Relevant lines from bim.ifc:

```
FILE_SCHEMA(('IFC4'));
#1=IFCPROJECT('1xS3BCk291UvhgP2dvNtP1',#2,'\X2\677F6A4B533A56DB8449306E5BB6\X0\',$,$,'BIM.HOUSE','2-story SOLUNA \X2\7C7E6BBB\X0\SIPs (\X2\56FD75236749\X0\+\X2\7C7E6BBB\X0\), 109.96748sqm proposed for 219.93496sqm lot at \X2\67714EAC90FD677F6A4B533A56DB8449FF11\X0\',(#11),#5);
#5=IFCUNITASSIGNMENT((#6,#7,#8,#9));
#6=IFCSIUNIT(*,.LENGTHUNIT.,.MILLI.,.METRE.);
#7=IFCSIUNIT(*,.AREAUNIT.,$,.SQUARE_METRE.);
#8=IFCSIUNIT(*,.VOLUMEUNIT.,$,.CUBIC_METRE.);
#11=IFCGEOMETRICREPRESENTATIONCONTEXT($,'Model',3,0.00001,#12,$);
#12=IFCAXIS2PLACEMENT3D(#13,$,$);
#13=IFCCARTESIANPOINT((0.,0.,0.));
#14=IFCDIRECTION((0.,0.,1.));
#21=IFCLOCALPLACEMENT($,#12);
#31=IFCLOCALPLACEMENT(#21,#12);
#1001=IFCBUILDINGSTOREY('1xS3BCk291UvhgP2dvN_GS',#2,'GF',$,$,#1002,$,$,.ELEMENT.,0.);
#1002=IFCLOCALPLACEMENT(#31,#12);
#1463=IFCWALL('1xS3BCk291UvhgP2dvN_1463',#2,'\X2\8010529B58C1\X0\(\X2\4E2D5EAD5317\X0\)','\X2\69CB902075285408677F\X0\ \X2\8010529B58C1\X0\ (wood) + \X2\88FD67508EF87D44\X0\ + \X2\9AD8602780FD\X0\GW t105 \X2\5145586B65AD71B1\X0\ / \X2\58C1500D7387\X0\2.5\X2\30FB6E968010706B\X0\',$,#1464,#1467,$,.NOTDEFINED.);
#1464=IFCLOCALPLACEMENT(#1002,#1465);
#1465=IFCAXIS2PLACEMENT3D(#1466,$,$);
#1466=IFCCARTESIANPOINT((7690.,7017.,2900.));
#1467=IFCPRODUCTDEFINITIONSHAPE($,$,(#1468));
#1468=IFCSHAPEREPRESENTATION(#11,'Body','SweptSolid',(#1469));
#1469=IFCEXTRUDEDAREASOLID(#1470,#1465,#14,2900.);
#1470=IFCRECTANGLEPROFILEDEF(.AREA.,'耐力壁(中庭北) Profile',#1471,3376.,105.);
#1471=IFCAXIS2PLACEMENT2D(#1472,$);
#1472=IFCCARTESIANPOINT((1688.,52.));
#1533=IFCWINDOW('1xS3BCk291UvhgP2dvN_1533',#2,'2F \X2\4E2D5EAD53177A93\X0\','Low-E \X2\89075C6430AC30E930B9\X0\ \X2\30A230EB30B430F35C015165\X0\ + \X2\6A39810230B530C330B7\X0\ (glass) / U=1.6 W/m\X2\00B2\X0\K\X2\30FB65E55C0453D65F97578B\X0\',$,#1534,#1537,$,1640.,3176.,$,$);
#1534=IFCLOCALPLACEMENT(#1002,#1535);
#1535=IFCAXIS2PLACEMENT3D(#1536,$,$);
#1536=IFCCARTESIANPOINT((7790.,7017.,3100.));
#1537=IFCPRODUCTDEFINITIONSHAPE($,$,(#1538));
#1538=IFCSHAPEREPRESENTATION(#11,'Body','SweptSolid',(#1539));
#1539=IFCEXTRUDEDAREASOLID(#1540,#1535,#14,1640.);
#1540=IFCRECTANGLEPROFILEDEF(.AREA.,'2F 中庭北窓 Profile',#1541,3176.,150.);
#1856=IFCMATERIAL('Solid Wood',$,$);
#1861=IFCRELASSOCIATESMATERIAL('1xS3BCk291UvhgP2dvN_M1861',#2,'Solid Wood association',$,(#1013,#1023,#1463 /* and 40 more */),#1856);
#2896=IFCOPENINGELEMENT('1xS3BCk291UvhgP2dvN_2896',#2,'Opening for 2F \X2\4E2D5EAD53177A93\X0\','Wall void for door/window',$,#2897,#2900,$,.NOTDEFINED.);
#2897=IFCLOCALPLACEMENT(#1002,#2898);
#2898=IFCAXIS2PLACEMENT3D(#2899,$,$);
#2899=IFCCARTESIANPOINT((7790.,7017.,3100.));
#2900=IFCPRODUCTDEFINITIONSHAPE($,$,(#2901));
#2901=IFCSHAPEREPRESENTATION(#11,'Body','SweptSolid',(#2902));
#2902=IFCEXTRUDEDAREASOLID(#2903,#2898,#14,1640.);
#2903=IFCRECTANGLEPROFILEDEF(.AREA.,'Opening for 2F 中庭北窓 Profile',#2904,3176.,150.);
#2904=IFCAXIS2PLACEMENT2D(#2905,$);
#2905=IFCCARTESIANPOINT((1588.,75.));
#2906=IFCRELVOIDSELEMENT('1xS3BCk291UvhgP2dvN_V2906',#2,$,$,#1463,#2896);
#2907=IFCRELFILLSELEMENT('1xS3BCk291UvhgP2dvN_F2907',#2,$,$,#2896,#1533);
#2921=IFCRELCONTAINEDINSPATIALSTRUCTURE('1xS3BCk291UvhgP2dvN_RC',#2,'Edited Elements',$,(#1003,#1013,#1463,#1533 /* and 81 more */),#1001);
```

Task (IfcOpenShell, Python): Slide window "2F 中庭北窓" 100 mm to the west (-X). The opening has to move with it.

```python
import ifcopenshell
import ifcopenshell.api.geometry
import ifcopenshell.util.placement

model = ifcopenshell.open("bim.ifc")

window = model.by_guid("1xS3BCk291UvhgP2dvN_1533")
opening = window.FillsVoids[0].RelatingOpeningElement
wall = opening.VoidsElements[0].RelatingBuildingElement

wall_matrix = ifcopenshell.util.placement.get_local_placement(wall.ObjectPlacement)
shift = wall_matrix[:3, 0] * -100.0
before = ifcopenshell.util.placement.get_local_placement(window.ObjectPlacement)[:3, 3].copy()

# The window is not placed relative to its opening, so move both.
for product in (opening, window):
    matrix = ifcopenshell.util.placement.get_local_placement(product.ObjectPlacement)
    matrix[:3, 3] += shift
    ifcopenshell.api.geometry.edit_object_placement(model, product=product, matrix=matrix, is_si=False)

after = ifcopenshell.util.placement.get_local_placement(window.ObjectPlacement)[:3, 3]
print("window moved by", (after - before).round(3) + 0.0)

model.write("bim_rev.ifc")
```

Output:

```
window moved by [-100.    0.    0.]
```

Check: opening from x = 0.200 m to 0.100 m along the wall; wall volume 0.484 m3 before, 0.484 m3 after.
